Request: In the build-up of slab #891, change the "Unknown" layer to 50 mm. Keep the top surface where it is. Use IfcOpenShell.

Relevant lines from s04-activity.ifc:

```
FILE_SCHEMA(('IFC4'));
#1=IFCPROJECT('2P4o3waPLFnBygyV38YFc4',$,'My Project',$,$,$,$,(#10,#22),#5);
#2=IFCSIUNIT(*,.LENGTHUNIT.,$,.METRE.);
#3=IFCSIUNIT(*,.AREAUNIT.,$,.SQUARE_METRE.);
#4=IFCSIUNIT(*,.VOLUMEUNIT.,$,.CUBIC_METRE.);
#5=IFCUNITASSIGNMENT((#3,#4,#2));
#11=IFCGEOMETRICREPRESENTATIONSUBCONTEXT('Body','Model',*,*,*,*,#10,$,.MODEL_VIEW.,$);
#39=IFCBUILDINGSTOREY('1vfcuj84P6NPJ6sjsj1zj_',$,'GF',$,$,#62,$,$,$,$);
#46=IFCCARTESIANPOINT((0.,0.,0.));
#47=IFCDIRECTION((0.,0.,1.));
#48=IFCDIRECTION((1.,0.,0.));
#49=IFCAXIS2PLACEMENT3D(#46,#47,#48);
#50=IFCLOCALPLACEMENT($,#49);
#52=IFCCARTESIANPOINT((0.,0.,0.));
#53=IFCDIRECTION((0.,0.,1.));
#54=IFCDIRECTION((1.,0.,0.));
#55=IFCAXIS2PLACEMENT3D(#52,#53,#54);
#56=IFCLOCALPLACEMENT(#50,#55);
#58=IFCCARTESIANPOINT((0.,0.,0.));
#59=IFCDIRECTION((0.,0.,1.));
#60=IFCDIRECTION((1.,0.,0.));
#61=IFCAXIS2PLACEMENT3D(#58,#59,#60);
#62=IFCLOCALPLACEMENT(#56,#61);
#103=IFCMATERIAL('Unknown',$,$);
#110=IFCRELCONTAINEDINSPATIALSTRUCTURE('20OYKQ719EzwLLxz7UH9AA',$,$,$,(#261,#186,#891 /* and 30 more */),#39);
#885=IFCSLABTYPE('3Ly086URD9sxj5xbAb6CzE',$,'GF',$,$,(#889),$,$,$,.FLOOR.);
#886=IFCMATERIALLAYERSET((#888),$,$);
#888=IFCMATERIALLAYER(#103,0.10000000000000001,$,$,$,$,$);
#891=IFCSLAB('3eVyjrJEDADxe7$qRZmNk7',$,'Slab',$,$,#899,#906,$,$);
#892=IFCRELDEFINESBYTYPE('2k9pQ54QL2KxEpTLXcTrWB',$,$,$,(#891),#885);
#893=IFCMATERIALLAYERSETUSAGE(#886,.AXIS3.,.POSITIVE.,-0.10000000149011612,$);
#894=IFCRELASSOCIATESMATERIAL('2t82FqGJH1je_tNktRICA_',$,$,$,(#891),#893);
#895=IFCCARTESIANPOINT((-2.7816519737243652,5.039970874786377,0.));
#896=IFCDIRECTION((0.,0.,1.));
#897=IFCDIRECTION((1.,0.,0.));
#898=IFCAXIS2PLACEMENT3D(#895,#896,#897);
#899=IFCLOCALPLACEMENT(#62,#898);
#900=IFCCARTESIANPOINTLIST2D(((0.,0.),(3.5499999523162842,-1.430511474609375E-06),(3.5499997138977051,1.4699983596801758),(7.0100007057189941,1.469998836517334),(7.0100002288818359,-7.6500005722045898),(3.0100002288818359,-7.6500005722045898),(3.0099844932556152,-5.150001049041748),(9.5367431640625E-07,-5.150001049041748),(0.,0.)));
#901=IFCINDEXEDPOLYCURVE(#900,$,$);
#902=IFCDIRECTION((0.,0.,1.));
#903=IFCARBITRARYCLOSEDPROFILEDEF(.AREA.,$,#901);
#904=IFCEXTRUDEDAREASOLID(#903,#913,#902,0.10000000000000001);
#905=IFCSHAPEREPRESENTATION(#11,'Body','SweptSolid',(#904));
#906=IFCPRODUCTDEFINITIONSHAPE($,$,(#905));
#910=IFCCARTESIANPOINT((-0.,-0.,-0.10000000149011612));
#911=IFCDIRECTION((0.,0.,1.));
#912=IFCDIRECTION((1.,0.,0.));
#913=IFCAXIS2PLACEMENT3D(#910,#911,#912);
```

```python
import ifcopenshell
import ifcopenshell.util.element
import ifcopenshell.util.representation
import ifcopenshell.util.unit

model = ifcopenshell.open("s04-activity.ifc")
unit_scale = ifcopenshell.util.unit.calculate_unit_scale(model)

layer_set = model.by_id(886)
layer = next(l for l in layer_set.MaterialLayers if l.Material and l.Material.Name == "Unknown")
change = 0.05 / unit_scale - layer.LayerThickness
layer.LayerThickness += change

# Geometry does not follow the layer set by itself.
slabs = [e for e in ifcopenshell.util.element.get_elements_by_material(model, layer_set) if e.is_a("IfcSlab")]
for slab in sorted(slabs, key=lambda e: e.id()):
    body = ifcopenshell.util.representation.get_representation(slab, "Model", "Body")
    solid = body.Items[0]
    old_depth = solid.Depth
    solid.Depth += change
    # Extruded upwards: lower the start of the extrusion so the top stays.
    x, y, z = solid.Position.Location.Coordinates
    solid.Position.Location = model.createIfcCartesianPoint((x, y, z - change))
    print(slab.id(), f"{old_depth:g} -> {solid.Depth:g}")

# The layers are counted up from the underside, which has moved.
for usage in {ifcopenshell.util.element.get_material(slab) for slab in slabs}:
    usage.OffsetFromReferenceLine -= change

model.write("s04-activity_edited.ifc")
```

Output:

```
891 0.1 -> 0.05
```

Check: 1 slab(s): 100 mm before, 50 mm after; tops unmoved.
